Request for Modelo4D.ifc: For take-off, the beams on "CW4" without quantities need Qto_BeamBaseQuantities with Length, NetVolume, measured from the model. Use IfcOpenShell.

First a look at what the model holds.

```python
import ifcopenshell
import ifcopenshell.util.element
import ifcopenshell.util.unit

model = ifcopenshell.open("Modelo4D.ifc")
print(model.schema)
for unit_type in ("LENGTHUNIT", "AREAUNIT", "VOLUMEUNIT"):
    print(unit_type, ifcopenshell.util.unit.calculate_unit_scale(model, unit_type))
storey = next(s for s in model.by_type("IfcBuildingStorey") if s.Name == "CW4")
beams = [e for e in ifcopenshell.util.element.get_decomposition(storey) if e.is_a("IfcBeam")]
for e in sorted(beams, key=lambda e: e.id()):
    print(e.id(), e.is_a(), e.Name, list(ifcopenshell.util.element.get_psets(e, qtos_only=True)), sep=" | ")
```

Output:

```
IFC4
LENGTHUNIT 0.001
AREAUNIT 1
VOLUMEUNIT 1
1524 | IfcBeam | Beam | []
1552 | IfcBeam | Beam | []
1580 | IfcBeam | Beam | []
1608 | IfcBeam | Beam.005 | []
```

```python
import ifcopenshell
import ifcopenshell.api.pset
import ifcopenshell.geom
import ifcopenshell.util.element
import ifcopenshell.util.shape
import ifcopenshell.util.unit

model = ifcopenshell.open("Modelo4D.ifc")
unit_scale = ifcopenshell.util.unit.calculate_unit_scale(model)
volume_scale = ifcopenshell.util.unit.calculate_unit_scale(model, "VOLUMEUNIT")
settings = ifcopenshell.geom.settings()

storey = next(s for s in model.by_type("IfcBuildingStorey") if s.Name == "CW4")
beams = [e for e in ifcopenshell.util.element.get_decomposition(storey) if e.is_a("IfcBeam")]

for e in sorted(beams, key=lambda e: e.id()):
    if ifcopenshell.util.element.get_psets(e, qtos_only=True, should_inherit=False):
        continue
    # Geometry comes back in metres, in the element's own axes.
    shape = ifcopenshell.geom.create_shape(settings, e)
    values = {
        "Length": ifcopenshell.util.shape.get_max_xyz(shape.geometry) / unit_scale,
        "NetVolume": ifcopenshell.util.shape.get_volume(shape.geometry) / volume_scale,
    }
    qto = ifcopenshell.api.pset.add_qto(model, product=e, name="Qto_BeamBaseQuantities")
    ifcopenshell.api.pset.edit_qto(model, qto=qto, properties=values)
    print(e.id(), {k: round(v, 3) for k, v in values.items()})

model.write("Modelo4D_updated.ifc")
```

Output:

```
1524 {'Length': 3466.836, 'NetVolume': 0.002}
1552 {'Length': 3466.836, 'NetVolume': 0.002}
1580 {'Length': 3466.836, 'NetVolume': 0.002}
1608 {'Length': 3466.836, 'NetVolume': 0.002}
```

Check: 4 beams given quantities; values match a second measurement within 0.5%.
